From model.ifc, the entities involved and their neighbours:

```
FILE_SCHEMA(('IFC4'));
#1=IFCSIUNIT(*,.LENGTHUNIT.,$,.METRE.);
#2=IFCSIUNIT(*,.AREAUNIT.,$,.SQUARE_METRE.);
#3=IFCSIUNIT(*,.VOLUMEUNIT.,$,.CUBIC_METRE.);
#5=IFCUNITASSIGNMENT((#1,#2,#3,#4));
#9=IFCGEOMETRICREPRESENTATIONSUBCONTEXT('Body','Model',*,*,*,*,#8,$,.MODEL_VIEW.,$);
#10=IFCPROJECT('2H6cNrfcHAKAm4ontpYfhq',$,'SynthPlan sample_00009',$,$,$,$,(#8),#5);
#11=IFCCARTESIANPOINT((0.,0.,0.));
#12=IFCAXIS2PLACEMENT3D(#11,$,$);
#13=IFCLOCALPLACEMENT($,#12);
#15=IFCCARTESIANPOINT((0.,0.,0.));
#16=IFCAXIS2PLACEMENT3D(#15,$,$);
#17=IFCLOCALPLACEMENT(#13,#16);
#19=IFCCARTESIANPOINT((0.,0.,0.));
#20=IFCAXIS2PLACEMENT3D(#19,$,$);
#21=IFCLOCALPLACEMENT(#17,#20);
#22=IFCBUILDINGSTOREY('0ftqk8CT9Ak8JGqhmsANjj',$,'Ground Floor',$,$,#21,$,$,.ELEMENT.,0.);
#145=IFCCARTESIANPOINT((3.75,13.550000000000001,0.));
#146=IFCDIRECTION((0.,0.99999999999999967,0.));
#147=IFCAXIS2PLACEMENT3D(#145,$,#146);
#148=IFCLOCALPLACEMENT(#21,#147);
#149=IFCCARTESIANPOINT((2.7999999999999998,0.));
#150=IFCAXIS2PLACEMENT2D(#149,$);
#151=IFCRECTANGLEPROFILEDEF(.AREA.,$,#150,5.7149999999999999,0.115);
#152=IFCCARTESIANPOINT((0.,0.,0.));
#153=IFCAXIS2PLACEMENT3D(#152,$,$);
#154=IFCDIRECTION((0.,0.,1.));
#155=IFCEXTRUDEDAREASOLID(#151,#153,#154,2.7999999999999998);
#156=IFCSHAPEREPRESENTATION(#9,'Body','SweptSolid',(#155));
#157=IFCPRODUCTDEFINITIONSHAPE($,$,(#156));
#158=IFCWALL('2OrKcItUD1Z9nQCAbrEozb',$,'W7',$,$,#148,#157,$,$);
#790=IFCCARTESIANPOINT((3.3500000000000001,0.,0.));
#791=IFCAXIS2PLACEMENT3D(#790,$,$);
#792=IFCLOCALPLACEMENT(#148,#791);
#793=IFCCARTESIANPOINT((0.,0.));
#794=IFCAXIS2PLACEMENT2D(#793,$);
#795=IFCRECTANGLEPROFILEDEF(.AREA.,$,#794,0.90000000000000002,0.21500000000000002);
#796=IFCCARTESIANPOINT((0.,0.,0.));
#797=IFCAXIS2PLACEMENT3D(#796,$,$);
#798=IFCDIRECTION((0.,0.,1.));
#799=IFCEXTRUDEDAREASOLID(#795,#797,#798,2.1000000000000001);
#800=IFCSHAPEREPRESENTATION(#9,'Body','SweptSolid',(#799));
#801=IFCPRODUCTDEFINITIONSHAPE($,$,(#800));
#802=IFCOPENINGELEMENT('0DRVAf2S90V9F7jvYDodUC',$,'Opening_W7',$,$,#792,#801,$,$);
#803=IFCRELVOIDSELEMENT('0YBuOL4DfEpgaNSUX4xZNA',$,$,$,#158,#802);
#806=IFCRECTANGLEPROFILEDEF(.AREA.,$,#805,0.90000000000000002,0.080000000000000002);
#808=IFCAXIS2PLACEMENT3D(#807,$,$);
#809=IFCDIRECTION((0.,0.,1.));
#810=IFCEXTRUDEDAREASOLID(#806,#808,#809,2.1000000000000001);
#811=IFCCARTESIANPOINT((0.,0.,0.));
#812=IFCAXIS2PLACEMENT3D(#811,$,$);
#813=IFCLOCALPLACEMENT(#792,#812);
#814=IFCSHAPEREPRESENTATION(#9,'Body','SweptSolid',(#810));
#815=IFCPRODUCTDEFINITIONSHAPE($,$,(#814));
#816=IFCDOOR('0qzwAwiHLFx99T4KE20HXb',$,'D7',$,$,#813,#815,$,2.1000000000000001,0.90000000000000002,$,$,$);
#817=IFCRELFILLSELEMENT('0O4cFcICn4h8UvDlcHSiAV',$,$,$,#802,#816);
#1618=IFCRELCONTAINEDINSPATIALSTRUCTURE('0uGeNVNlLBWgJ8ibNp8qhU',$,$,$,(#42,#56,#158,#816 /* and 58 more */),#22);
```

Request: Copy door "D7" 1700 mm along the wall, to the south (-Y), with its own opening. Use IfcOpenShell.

```python
import ifcopenshell
import ifcopenshell.api.feature
import ifcopenshell.api.geometry
import ifcopenshell.api.root
import ifcopenshell.geom
import ifcopenshell.util.element
import ifcopenshell.util.placement
import ifcopenshell.util.shape
import ifcopenshell.util.unit

model = ifcopenshell.open("model.ifc")
unit_scale = ifcopenshell.util.unit.calculate_unit_scale(model)
settings = ifcopenshell.geom.settings()


def volume(element):
    """Net volume in cubic metres, openings subtracted."""
    shape = ifcopenshell.geom.create_shape(settings, element)
    return ifcopenshell.util.shape.get_volume(shape.geometry)


door = model.by_id(816)
opening = door.FillsVoids[0].RelatingOpeningElement
wall = opening.VoidsElements[0].RelatingBuildingElement
before = volume(wall)
shift = ifcopenshell.util.placement.get_local_placement(wall.ObjectPlacement)[:3, 0] * -1.7 / unit_scale

# copy_class copies the void relationship, type, container and properties, but no geometry.
new_opening = ifcopenshell.api.root.copy_class(model, product=opening)
new_opening.Representation = ifcopenshell.util.element.copy_deep(
    model, opening.Representation, exclude=["IfcGeometricRepresentationContext", "IfcRepresentationMap"]
)
new_door = ifcopenshell.api.root.copy_class(model, product=door)
new_door.Representation = ifcopenshell.util.element.copy_deep(
    model, door.Representation, exclude=["IfcGeometricRepresentationContext", "IfcRepresentationMap"]
)
ifcopenshell.api.feature.add_filling(model, opening=new_opening, element=new_door)

for old, new in ((opening, new_opening), (door, new_door)):
    matrix = ifcopenshell.util.placement.get_local_placement(old.ObjectPlacement)
    matrix[:3, 3] += shift
    ifcopenshell.api.geometry.edit_object_placement(model, product=new, matrix=matrix, is_si=False)

after = volume(wall)

print(f"wall volume {before:.3f} -> {after:.3f} m3")

model.write("model_edited.ifc")
```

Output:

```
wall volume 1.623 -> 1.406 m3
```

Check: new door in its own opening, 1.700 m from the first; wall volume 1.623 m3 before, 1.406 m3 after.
